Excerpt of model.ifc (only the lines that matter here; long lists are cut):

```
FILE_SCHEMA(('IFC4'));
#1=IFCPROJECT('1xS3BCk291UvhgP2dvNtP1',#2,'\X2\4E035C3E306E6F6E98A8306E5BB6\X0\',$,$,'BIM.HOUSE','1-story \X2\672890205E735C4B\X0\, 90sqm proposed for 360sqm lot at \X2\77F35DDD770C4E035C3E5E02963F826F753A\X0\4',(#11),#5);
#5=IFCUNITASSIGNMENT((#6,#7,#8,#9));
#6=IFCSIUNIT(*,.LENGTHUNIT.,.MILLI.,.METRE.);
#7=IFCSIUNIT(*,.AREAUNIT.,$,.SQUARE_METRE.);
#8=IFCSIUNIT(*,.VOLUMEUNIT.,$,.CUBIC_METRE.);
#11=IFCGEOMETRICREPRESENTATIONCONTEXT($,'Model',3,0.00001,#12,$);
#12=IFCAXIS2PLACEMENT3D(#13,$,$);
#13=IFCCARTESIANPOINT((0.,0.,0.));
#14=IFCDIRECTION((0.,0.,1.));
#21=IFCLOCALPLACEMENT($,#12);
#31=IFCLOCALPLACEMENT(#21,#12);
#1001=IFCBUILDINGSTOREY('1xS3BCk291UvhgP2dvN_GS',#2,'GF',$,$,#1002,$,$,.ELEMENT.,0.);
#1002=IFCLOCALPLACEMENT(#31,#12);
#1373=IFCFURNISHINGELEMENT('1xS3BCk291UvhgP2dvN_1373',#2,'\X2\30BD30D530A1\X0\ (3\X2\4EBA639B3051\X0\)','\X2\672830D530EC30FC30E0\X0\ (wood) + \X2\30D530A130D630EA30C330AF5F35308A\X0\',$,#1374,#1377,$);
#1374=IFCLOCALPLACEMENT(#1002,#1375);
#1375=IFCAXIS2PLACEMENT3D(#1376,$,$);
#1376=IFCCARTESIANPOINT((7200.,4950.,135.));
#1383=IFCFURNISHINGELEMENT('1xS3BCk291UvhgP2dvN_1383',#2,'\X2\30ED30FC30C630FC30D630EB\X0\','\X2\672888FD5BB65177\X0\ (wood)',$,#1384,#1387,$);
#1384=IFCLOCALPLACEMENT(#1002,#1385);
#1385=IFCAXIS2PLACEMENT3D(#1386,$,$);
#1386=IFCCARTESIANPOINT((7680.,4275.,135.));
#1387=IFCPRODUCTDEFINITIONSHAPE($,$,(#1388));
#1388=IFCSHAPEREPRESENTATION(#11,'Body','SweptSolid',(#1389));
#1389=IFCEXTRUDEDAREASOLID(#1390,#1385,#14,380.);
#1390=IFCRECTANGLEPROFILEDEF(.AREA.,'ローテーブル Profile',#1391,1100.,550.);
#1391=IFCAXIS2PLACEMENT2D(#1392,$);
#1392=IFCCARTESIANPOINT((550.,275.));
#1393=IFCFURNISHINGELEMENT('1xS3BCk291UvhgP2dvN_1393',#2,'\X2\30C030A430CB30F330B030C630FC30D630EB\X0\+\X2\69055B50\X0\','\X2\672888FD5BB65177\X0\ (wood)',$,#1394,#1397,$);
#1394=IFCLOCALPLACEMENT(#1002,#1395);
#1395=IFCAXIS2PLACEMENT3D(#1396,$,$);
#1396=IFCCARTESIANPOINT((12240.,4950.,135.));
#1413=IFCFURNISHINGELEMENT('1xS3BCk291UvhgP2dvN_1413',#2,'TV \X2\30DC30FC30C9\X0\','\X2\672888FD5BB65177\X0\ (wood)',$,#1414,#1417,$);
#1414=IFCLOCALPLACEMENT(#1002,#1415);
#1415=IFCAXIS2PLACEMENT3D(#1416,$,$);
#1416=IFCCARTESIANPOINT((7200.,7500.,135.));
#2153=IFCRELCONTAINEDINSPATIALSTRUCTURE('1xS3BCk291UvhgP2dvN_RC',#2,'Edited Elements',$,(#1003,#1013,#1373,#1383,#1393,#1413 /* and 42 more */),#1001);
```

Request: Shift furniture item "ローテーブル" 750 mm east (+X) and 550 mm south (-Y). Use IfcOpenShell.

```python
import ifcopenshell
import ifcopenshell.api.geometry
import ifcopenshell.util.placement
import ifcopenshell.util.unit

model = ifcopenshell.open("model.ifc")
unit_scale = ifcopenshell.util.unit.calculate_unit_scale(model)

item = model.by_id(1383)
matrix = ifcopenshell.util.placement.get_local_placement(item.ObjectPlacement)
matrix[0, 3] += 0.75 / unit_scale
matrix[1, 3] -= 0.55 / unit_scale
ifcopenshell.api.geometry.edit_object_placement(model, product=item, matrix=matrix, is_si=False)

print(ifcopenshell.util.placement.get_local_placement(item.ObjectPlacement).round(3) + 0.0)

model.write("model_updated.ifc")
```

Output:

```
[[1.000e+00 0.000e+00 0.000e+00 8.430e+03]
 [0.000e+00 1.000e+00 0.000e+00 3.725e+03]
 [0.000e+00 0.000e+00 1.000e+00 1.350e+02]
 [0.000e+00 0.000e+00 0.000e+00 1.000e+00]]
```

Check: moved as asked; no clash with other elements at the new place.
